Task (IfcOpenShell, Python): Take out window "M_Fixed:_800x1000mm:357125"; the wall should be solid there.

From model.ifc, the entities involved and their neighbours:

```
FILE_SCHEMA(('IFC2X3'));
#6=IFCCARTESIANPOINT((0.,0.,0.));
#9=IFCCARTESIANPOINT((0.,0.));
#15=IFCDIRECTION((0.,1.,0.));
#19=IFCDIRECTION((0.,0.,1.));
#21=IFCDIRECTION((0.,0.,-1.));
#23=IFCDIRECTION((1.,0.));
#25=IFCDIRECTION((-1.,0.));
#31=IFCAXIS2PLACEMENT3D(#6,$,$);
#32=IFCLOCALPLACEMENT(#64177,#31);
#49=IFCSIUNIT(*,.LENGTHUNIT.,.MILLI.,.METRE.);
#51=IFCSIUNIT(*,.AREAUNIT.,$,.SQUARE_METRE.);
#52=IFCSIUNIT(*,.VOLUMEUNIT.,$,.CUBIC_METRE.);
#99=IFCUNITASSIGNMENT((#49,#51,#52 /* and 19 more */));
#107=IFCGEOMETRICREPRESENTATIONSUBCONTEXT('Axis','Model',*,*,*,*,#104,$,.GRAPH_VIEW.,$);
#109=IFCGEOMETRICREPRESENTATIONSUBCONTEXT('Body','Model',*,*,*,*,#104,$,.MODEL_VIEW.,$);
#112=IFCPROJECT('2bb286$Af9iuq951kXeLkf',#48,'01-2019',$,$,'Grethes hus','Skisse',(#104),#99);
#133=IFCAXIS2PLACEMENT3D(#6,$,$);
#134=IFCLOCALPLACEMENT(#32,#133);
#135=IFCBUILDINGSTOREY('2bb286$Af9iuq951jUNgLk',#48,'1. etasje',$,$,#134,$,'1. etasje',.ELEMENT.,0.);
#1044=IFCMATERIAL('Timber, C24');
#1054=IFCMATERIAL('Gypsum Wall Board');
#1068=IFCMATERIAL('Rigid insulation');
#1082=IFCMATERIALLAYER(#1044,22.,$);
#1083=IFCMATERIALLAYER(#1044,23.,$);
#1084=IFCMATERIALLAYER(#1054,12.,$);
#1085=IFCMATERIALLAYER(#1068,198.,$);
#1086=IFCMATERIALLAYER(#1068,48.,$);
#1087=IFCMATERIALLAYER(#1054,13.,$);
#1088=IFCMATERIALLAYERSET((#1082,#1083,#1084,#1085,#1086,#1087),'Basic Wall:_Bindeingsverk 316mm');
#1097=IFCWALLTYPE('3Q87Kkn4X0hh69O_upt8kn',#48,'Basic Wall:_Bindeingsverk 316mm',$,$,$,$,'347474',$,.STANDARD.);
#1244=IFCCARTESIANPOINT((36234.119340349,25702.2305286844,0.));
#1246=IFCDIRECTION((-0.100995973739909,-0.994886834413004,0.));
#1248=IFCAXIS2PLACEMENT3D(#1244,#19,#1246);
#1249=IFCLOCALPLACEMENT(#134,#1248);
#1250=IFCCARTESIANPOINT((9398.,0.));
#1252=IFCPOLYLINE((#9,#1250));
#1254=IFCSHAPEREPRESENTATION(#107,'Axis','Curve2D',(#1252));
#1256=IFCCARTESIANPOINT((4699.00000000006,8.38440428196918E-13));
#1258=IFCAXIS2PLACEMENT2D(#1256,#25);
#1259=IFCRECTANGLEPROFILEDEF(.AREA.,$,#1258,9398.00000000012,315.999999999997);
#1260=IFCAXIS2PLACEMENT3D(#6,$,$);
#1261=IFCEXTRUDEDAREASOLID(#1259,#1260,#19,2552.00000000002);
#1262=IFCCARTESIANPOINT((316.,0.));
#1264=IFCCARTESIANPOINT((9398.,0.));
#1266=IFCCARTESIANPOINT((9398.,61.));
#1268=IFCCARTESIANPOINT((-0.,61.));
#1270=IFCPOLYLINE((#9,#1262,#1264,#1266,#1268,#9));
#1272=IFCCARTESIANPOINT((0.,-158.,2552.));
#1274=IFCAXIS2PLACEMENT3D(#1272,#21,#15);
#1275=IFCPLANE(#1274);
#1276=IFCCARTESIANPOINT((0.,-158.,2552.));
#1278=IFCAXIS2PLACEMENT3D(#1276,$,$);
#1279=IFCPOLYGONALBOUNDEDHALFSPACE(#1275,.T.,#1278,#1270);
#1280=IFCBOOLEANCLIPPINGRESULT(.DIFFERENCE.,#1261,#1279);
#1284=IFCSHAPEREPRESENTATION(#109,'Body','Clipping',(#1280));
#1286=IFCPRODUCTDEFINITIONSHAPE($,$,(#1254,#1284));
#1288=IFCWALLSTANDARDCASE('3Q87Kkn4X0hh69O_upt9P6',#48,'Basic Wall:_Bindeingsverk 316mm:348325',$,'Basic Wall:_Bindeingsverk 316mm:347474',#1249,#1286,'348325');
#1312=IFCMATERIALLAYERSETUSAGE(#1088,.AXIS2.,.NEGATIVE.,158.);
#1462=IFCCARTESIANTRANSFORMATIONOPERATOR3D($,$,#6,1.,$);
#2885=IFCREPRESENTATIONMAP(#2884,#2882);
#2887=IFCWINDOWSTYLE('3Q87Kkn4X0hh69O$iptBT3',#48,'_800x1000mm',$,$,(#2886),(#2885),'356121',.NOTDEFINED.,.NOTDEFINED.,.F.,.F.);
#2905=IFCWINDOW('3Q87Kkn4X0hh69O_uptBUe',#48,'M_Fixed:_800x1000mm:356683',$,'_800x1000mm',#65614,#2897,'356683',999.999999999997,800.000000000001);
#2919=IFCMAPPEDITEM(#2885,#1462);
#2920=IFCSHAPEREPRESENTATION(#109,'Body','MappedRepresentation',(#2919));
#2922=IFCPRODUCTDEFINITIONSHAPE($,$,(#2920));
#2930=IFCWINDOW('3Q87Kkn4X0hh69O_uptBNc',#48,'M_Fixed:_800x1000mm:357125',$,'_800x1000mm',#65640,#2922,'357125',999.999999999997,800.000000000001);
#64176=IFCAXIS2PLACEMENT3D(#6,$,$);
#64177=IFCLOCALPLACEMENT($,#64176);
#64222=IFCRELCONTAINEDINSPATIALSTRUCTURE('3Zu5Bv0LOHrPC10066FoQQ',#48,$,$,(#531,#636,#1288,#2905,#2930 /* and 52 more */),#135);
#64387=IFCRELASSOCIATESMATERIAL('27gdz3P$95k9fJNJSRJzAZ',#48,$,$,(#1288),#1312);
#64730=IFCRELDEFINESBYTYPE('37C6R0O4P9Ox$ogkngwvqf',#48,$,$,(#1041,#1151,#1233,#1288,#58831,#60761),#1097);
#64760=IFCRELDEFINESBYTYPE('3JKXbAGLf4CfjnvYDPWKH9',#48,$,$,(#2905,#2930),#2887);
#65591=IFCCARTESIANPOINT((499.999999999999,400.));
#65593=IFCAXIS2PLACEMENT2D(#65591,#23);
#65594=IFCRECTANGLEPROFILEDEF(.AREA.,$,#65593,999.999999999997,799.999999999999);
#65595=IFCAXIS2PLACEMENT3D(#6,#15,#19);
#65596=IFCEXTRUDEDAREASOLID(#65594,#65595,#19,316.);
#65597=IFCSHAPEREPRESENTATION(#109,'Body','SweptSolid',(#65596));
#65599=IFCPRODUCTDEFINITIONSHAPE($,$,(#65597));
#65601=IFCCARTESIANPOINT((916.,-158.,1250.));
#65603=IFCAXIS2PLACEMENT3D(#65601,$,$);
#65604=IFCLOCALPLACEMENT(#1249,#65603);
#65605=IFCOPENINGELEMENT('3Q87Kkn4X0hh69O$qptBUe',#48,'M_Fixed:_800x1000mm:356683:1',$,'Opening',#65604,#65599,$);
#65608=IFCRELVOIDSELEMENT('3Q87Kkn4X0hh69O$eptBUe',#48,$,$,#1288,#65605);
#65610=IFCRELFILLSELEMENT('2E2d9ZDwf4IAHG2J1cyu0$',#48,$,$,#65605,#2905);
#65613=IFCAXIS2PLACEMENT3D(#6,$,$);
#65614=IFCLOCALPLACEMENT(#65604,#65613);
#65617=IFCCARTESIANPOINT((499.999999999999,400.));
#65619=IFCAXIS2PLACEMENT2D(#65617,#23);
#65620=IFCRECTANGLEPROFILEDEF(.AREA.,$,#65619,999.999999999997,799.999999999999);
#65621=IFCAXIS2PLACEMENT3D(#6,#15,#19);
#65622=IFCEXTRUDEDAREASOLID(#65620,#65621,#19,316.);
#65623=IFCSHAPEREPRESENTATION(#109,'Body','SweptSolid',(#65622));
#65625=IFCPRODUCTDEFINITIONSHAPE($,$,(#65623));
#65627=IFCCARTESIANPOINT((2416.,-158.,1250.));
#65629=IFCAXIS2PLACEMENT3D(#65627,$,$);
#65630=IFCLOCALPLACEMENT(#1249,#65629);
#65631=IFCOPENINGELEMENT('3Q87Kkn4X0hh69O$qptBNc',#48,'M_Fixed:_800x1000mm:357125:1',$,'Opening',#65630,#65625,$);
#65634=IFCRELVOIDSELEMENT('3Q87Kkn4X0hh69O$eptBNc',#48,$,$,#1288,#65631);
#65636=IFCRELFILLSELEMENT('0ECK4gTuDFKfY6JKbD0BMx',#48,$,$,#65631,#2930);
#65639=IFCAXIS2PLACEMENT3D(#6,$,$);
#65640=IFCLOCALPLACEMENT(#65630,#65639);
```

```python
import ifcopenshell
import ifcopenshell.api.feature
import ifcopenshell.api.root
import ifcopenshell.geom
import ifcopenshell.util.shape

model = ifcopenshell.open("model.ifc")
settings = ifcopenshell.geom.settings()


def volume(element):
    """Net volume in cubic metres, openings subtracted."""
    shape = ifcopenshell.geom.create_shape(settings, element)
    return ifcopenshell.util.shape.get_volume(shape.geometry)


window = model.by_guid("3Q87Kkn4X0hh69O_uptBNc")
opening = window.FillsVoids[0].RelatingOpeningElement
wall = opening.VoidsElements[0].RelatingBuildingElement
before = volume(wall)

ifcopenshell.api.root.remove_product(model, product=window)
ifcopenshell.api.feature.remove_feature(model, feature=opening)

after = volume(wall)

print(f"wall volume {before:.3f} -> {after:.3f} m3")

model.write("model_v2.ifc")
```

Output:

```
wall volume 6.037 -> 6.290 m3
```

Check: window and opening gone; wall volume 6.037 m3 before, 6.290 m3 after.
